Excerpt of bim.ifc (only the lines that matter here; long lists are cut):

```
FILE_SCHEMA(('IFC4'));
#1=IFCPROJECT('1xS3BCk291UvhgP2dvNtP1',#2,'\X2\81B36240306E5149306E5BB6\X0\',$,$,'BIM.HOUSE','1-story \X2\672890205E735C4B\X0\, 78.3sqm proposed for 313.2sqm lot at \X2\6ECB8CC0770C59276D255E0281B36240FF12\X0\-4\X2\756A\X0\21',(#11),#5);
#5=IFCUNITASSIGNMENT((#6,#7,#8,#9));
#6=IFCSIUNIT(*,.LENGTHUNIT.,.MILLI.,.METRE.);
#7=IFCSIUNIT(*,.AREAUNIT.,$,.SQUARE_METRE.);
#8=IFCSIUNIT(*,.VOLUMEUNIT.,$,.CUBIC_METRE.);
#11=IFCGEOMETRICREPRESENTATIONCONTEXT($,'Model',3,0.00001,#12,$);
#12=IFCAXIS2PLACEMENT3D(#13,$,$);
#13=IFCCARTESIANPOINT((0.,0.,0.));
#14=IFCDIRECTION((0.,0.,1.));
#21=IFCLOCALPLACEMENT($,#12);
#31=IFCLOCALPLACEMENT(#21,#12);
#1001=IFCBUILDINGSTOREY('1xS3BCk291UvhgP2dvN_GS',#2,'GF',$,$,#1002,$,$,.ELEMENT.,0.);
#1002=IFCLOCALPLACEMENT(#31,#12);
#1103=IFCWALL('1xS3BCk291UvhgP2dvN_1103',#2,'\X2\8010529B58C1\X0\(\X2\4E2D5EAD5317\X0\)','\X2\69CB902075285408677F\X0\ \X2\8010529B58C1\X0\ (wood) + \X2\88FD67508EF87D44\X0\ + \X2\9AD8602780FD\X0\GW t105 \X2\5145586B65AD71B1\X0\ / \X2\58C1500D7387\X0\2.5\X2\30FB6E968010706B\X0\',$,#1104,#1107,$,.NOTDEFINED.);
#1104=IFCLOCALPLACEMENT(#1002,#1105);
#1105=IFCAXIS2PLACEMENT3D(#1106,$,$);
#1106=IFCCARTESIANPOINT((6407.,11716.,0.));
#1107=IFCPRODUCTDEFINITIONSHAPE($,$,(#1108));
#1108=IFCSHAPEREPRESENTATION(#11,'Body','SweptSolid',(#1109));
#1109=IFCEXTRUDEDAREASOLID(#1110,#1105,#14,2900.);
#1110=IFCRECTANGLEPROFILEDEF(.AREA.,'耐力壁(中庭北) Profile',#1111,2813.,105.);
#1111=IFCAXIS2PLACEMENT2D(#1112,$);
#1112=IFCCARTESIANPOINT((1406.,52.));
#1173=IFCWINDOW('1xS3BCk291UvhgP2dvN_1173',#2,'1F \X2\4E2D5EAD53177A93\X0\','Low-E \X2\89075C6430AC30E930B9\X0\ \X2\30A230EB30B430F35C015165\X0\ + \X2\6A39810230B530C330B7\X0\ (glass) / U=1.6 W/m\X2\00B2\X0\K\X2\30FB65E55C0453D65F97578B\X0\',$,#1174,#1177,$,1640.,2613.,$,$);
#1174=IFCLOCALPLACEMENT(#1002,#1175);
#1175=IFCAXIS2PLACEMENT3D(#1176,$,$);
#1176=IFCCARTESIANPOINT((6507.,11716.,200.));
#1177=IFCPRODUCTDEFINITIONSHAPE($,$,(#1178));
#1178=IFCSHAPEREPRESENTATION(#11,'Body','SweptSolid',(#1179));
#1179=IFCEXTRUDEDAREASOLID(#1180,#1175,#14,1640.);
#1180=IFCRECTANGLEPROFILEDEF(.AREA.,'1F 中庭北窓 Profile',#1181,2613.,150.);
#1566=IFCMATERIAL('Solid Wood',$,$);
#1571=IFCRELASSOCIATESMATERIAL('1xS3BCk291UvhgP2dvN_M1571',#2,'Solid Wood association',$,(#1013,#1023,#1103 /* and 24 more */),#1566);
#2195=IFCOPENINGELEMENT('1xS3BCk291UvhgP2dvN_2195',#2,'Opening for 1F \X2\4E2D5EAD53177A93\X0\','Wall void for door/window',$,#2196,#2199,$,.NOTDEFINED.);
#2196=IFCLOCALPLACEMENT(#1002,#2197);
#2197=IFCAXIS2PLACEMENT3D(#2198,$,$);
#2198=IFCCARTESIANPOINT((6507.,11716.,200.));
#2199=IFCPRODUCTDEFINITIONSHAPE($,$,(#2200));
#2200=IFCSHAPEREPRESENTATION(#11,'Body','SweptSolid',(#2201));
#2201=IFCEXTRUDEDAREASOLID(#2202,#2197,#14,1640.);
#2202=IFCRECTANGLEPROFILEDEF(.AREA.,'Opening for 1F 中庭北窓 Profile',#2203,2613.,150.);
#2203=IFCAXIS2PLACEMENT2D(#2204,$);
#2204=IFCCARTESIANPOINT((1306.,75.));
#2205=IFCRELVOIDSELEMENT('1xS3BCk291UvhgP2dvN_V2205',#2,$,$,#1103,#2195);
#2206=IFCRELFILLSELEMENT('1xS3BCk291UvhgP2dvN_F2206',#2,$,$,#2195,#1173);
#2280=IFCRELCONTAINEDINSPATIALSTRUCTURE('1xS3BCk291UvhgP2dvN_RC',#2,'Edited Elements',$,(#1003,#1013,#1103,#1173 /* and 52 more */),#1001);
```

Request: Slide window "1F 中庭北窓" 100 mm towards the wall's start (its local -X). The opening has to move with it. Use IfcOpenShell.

```python
import ifcopenshell
import ifcopenshell.api.geometry
import ifcopenshell.util.placement
import ifcopenshell.util.unit

model = ifcopenshell.open("bim.ifc")
unit_scale = ifcopenshell.util.unit.calculate_unit_scale(model)

window = model.by_guid("1xS3BCk291UvhgP2dvN_1173")
opening = window.FillsVoids[0].RelatingOpeningElement
wall = opening.VoidsElements[0].RelatingBuildingElement

wall_matrix = ifcopenshell.util.placement.get_local_placement(wall.ObjectPlacement)
shift = wall_matrix[:3, 0] * -0.1 / unit_scale
before = ifcopenshell.util.placement.get_local_placement(window.ObjectPlacement)[:3, 3].copy()

# The window is not placed relative to its opening, so move both.
for product in (opening, window):
    matrix = ifcopenshell.util.placement.get_local_placement(product.ObjectPlacement)
    matrix[:3, 3] += shift
    ifcopenshell.api.geometry.edit_object_placement(model, product=product, matrix=matrix, is_si=False)

after = ifcopenshell.util.placement.get_local_placement(window.ObjectPlacement)[:3, 3]
print("window moved by", (after - before).round(3) + 0.0)

model.write("bim-out.ifc")
```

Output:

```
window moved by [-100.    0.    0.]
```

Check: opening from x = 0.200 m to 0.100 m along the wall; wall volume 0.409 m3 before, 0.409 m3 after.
